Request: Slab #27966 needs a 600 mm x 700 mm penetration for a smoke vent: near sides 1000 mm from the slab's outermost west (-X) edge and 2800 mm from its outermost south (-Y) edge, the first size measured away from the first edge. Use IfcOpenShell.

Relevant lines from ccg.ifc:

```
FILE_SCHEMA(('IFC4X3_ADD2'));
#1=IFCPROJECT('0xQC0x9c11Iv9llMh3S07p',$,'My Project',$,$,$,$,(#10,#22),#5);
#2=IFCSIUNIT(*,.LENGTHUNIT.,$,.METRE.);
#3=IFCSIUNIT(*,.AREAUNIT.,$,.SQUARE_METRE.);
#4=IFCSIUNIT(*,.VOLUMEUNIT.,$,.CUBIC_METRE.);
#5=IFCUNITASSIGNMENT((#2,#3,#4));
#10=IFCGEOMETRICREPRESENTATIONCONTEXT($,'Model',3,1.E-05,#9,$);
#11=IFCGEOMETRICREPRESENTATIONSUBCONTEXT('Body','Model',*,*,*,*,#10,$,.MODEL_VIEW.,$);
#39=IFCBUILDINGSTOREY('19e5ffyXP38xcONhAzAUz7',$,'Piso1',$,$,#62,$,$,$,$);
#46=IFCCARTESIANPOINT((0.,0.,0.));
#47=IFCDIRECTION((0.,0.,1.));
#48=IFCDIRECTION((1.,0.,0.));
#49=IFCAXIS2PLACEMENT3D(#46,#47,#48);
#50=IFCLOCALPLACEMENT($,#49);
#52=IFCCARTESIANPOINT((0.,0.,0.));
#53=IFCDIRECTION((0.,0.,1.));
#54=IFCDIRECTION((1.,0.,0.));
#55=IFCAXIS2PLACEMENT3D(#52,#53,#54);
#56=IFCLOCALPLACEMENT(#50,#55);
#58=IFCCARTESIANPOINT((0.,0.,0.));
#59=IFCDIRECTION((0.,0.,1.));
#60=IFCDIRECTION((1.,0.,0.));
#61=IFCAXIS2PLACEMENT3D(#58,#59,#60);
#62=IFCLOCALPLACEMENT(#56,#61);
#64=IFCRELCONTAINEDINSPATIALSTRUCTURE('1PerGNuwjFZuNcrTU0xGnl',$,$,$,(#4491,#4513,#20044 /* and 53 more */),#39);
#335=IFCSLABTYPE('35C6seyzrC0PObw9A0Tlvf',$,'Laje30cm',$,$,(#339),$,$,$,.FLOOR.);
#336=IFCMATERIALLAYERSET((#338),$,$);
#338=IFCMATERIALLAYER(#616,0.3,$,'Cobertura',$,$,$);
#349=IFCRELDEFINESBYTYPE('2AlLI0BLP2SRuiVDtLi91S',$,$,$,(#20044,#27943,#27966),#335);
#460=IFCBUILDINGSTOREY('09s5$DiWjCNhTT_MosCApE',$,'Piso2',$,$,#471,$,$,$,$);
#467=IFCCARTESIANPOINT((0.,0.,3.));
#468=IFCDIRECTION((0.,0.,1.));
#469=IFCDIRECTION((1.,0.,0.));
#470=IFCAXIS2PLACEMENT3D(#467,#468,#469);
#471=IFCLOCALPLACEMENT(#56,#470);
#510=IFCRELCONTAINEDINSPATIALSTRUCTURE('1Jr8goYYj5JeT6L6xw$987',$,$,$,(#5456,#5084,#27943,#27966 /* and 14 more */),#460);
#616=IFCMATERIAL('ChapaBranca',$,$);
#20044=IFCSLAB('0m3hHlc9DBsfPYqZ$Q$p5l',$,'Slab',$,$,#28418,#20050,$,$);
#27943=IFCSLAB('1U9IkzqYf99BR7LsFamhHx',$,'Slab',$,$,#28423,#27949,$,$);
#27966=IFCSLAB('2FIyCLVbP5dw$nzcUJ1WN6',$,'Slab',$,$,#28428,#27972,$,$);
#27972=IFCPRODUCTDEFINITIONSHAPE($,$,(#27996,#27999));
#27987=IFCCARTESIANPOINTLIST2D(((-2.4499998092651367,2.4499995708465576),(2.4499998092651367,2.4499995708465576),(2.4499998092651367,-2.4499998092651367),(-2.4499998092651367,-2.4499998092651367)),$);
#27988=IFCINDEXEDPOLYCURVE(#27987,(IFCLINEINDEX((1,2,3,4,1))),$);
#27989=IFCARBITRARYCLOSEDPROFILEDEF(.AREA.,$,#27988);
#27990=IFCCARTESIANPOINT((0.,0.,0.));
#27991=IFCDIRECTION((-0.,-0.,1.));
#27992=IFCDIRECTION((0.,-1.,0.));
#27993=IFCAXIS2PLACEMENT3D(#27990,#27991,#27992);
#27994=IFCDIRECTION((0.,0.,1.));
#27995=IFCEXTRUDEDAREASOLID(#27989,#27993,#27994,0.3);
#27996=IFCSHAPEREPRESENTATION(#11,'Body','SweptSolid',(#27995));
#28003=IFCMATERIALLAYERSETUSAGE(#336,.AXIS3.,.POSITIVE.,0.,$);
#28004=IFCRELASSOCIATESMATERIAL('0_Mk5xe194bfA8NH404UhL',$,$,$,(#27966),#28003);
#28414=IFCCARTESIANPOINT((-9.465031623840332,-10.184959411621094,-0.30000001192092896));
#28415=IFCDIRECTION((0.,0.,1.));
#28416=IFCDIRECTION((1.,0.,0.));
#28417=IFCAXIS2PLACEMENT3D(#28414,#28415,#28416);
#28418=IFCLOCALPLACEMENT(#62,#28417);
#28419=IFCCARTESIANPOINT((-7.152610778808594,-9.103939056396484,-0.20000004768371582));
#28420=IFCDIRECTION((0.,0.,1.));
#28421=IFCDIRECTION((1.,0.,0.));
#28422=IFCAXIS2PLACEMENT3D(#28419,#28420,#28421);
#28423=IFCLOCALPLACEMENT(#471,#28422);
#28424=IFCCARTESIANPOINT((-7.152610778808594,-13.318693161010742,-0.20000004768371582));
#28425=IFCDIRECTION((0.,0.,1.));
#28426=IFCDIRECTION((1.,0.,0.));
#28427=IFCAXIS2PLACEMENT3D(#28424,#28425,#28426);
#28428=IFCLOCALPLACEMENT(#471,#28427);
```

```python
import numpy as np
import ifcopenshell
import ifcopenshell.api.feature
import ifcopenshell.api.geometry
import ifcopenshell.api.root
import ifcopenshell.geom
import ifcopenshell.util.placement
import ifcopenshell.util.representation
import ifcopenshell.util.shape
import ifcopenshell.util.unit

model = ifcopenshell.open("ccg.ifc")
unit_scale = ifcopenshell.util.unit.calculate_unit_scale(model)
settings = ifcopenshell.geom.settings()


def volume(element):
    """Net volume in cubic metres, openings subtracted."""
    shape = ifcopenshell.geom.create_shape(settings, element)
    return ifcopenshell.util.shape.get_volume(shape.geometry)


slab = model.by_guid("2FIyCLVbP5dw$nzcUJ1WN6")
before = volume(slab)

# Extent in the slab's own axes, in metres. The edges named are its -X and -Y sides.
slab_shape = ifcopenshell.geom.create_shape(settings, slab)
vertices = ifcopenshell.util.shape.get_vertices(slab_shape.geometry)
x_min, y_min, bottom = vertices.min(axis=0)
top = vertices[:, 2].max()

opening = ifcopenshell.api.root.create_entity(model, ifc_class="IfcOpeningElement", name="Smoke vent opening", predefined_type="OPENING")
context = ifcopenshell.util.representation.get_context(model, "Model", "Body", "MODEL_VIEW")
width, depth = 0.6, 0.7
outline = [(0.0, 0.0), (width, 0.0), (width, depth), (0.0, depth), (0.0, 0.0)]
# Overshoot both faces by 50 mm so the cut is clean.
shape = ifcopenshell.api.geometry.add_slab_representation(
    model, context=context, depth=top - bottom + 0.1, polyline=outline
)
ifcopenshell.api.geometry.assign_representation(model, product=opening, representation=shape)

matrix = ifcopenshell.util.placement.get_local_placement(slab.ObjectPlacement)
matrix[:, 3] = matrix @ np.append(np.array([x_min + 1, y_min + 2.8, bottom - 0.05]) / unit_scale, 1.0)
ifcopenshell.api.geometry.edit_object_placement(model, product=opening, matrix=matrix, is_si=False)
ifcopenshell.api.feature.add_feature(model, feature=opening, element=slab)

after = volume(slab)

print(f"slab volume {before:.3f} -> {after:.3f} m3")

model.write("ccg_updated.ifc")
```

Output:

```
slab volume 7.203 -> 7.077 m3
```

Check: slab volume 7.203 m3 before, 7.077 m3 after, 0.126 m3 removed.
